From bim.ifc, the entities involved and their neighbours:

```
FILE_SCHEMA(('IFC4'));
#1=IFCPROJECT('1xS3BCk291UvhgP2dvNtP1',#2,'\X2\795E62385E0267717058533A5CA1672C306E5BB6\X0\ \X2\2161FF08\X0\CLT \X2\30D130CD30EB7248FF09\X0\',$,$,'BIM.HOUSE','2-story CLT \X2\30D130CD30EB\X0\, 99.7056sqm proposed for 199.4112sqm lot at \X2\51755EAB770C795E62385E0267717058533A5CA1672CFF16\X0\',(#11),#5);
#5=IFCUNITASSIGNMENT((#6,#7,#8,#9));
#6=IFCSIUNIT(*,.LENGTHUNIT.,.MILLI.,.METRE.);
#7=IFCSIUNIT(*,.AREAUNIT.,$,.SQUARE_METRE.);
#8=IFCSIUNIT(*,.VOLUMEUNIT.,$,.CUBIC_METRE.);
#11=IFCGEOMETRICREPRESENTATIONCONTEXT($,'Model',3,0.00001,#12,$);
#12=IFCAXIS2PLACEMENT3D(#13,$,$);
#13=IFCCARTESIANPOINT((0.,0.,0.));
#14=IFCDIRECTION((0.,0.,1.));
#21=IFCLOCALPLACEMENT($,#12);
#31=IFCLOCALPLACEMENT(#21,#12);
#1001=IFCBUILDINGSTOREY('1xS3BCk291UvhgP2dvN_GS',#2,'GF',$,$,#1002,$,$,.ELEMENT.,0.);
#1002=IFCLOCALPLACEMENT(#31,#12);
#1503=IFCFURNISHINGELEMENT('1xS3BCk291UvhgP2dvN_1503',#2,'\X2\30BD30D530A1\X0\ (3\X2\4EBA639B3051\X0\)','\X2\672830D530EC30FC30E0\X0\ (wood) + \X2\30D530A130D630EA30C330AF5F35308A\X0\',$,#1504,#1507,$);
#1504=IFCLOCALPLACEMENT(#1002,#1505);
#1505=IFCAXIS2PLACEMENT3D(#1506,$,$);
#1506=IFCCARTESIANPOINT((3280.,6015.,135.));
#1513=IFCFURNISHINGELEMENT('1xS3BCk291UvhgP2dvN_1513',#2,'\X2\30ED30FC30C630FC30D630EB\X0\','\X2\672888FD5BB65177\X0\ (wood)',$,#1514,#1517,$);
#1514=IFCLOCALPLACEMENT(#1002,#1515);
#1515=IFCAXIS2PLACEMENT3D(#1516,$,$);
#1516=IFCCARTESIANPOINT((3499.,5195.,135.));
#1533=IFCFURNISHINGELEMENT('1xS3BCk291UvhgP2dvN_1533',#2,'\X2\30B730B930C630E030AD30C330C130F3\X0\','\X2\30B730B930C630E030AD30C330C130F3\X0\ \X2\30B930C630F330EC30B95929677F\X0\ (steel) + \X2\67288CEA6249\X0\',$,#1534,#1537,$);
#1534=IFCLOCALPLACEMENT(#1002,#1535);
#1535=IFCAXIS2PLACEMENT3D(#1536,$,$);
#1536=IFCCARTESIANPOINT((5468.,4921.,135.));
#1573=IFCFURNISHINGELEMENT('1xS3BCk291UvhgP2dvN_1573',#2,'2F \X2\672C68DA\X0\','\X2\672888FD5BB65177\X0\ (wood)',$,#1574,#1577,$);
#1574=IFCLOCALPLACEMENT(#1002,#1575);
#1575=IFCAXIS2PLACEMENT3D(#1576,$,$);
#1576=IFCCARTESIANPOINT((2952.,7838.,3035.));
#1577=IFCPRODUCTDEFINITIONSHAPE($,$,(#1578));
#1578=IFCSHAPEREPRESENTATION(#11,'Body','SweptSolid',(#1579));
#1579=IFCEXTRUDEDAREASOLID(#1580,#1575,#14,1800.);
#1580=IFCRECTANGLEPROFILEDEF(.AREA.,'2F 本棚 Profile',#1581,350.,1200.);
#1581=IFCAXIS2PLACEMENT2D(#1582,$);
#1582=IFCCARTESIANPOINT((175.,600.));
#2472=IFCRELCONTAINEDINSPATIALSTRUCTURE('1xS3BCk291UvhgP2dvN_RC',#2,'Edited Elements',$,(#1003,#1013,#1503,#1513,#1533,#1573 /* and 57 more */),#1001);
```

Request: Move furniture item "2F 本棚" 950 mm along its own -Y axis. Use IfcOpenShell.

```python
import ifcopenshell
import ifcopenshell.api.geometry
import ifcopenshell.util.placement
import ifcopenshell.util.unit

model = ifcopenshell.open("bim.ifc")
unit_scale = ifcopenshell.util.unit.calculate_unit_scale(model)

item = model.by_id(1573)
matrix = ifcopenshell.util.placement.get_local_placement(item.ObjectPlacement)
matrix[:3, 3] -= matrix[:3, 1] * 0.95 / unit_scale
ifcopenshell.api.geometry.edit_object_placement(model, product=item, matrix=matrix, is_si=False)

print(ifcopenshell.util.placement.get_local_placement(item.ObjectPlacement).round(3) + 0.0)

model.write("bim_rev.ifc")
```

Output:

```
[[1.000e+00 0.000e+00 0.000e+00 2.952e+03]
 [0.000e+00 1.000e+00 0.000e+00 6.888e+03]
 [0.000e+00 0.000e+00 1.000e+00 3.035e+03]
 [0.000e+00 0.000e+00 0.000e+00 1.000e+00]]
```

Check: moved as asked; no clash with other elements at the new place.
